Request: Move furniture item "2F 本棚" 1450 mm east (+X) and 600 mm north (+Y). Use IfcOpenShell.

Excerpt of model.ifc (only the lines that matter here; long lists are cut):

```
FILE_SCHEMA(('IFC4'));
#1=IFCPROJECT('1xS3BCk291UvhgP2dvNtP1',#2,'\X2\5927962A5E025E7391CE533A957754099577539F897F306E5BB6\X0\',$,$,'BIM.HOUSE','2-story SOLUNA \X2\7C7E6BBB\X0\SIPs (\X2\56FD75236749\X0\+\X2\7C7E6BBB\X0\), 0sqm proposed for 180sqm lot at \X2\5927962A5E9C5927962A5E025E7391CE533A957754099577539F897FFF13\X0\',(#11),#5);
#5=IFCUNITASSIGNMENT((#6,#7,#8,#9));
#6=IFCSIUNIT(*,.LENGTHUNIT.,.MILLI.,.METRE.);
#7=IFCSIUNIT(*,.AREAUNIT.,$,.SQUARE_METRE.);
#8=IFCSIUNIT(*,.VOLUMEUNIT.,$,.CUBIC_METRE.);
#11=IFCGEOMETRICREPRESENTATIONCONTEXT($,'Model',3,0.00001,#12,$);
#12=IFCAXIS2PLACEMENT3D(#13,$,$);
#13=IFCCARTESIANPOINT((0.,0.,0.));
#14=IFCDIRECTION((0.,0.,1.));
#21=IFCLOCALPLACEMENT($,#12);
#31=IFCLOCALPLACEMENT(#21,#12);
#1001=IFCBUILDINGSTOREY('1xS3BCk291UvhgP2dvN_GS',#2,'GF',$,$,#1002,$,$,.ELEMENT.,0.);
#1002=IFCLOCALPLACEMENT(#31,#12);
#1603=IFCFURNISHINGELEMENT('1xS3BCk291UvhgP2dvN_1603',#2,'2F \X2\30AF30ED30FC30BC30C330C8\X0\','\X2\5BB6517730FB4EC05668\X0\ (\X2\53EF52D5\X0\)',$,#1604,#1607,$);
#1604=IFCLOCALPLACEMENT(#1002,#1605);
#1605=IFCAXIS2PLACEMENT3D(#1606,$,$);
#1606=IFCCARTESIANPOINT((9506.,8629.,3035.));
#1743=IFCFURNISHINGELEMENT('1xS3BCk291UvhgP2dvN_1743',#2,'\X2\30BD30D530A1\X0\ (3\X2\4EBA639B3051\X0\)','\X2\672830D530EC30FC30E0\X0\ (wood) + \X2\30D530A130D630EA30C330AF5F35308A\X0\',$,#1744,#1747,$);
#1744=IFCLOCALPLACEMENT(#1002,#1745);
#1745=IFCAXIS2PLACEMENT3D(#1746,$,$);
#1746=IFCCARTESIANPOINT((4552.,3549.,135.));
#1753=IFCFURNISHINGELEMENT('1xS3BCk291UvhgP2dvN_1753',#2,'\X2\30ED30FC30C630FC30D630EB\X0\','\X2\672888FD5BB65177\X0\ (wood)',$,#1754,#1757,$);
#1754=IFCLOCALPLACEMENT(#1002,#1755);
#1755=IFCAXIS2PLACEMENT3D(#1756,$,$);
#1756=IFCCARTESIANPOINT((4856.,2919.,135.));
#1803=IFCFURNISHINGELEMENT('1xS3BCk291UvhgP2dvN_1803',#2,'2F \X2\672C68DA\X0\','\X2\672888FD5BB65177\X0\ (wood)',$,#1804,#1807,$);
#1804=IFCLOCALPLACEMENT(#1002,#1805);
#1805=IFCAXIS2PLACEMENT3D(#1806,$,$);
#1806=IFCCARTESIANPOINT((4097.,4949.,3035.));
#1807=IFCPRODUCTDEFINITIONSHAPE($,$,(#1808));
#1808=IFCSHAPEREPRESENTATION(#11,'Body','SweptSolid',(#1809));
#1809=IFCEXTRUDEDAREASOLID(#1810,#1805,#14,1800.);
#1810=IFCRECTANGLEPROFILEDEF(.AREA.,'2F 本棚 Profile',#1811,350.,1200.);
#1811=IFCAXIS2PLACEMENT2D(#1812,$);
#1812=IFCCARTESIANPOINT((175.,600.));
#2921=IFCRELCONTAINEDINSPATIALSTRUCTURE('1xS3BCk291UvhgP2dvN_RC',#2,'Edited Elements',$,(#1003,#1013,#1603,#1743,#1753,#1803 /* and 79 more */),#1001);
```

```python
import ifcopenshell
import ifcopenshell.api.geometry
import ifcopenshell.util.placement
import ifcopenshell.util.unit

model = ifcopenshell.open("model.ifc")
unit_scale = ifcopenshell.util.unit.calculate_unit_scale(model)

item = model.by_guid("1xS3BCk291UvhgP2dvN_1803")
matrix = ifcopenshell.util.placement.get_local_placement(item.ObjectPlacement)
matrix[0, 3] += 1.45 / unit_scale
matrix[1, 3] += 0.6 / unit_scale
ifcopenshell.api.geometry.edit_object_placement(model, product=item, matrix=matrix, is_si=False)

print(ifcopenshell.util.placement.get_local_placement(item.ObjectPlacement).round(3) + 0.0)

model.write("model_edited.ifc")
```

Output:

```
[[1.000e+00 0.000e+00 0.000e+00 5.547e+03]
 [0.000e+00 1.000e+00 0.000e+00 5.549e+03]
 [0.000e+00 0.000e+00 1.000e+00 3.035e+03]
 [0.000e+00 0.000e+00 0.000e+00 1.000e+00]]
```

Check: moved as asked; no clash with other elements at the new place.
